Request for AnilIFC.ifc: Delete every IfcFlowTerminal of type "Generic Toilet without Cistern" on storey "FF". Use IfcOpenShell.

First a look at what the model holds.

```python
import ifcopenshell
import ifcopenshell.util.element

model = ifcopenshell.open("AnilIFC.ifc")
print(model.schema)
storey = next(s for s in model.by_type("IfcBuildingStorey") if s.Name == "FF")
terminals = [e for e in ifcopenshell.util.element.get_decomposition(storey) if e.is_a("IfcFlowTerminal")]
seen = {}
for e in terminals:
    element_type = ifcopenshell.util.element.get_type(e)
    name = element_type.Name if element_type not in (None, e) else None
    seen[name] = seen.get(name, 0) + 1
for name, count in sorted(seen.items(), key=str):
    print(count, "x", name)
```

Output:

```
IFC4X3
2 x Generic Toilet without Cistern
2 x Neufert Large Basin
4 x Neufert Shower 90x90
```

```python
import ifcopenshell
import ifcopenshell.api.root
import ifcopenshell.util.element

model = ifcopenshell.open("AnilIFC.ifc")

storey = next(s for s in model.by_type("IfcBuildingStorey") if s.Name == "FF")
terminals = [e for e in ifcopenshell.util.element.get_decomposition(storey) if e.is_a("IfcFlowTerminal")]
targets = [e for e in terminals if (t := ifcopenshell.util.element.get_type(e)) not in (None, e) and t.Name == "Generic Toilet without Cistern"]

for e in targets:
    ifcopenshell.api.root.remove_product(model, product=e)
print(len(targets), "removed")

model.write("AnilIFC_edited.ifc")
```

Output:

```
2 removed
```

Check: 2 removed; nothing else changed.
